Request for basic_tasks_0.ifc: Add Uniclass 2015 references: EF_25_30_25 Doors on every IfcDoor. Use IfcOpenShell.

First a look at what the model holds.

```python
import ifcopenshell

model = ifcopenshell.open("basic_tasks_0.ifc")
print(model.schema)
print("classifications:", [c.Name for c in model.by_type("IfcClassification")])
for ifc_class in ("IfcDoor", "IfcRoof", "IfcStair", "IfcWall", "IfcWindow"):
    print(ifc_class, len(model.by_type(ifc_class)))
```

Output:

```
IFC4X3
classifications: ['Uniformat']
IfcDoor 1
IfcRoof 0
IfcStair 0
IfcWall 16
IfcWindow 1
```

```python
import ifcopenshell
import ifcopenshell.api.classification

model = ifcopenshell.open("basic_tasks_0.ifc")

system = ifcopenshell.api.classification.add_classification(model, classification="Uniclass 2015")

codes = {
    "IfcDoor": ("EF_25_30_25", "Doors"),
}
for ifc_class, (code, name) in codes.items():
    products = model.by_type(ifc_class)
    ifcopenshell.api.classification.add_reference(
        model, products=products, classification=system, identification=code, name=name
    )
    print(code, len(products))

model.write("basic_tasks_0-out.ifc")
```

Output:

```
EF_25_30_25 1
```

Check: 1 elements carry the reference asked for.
